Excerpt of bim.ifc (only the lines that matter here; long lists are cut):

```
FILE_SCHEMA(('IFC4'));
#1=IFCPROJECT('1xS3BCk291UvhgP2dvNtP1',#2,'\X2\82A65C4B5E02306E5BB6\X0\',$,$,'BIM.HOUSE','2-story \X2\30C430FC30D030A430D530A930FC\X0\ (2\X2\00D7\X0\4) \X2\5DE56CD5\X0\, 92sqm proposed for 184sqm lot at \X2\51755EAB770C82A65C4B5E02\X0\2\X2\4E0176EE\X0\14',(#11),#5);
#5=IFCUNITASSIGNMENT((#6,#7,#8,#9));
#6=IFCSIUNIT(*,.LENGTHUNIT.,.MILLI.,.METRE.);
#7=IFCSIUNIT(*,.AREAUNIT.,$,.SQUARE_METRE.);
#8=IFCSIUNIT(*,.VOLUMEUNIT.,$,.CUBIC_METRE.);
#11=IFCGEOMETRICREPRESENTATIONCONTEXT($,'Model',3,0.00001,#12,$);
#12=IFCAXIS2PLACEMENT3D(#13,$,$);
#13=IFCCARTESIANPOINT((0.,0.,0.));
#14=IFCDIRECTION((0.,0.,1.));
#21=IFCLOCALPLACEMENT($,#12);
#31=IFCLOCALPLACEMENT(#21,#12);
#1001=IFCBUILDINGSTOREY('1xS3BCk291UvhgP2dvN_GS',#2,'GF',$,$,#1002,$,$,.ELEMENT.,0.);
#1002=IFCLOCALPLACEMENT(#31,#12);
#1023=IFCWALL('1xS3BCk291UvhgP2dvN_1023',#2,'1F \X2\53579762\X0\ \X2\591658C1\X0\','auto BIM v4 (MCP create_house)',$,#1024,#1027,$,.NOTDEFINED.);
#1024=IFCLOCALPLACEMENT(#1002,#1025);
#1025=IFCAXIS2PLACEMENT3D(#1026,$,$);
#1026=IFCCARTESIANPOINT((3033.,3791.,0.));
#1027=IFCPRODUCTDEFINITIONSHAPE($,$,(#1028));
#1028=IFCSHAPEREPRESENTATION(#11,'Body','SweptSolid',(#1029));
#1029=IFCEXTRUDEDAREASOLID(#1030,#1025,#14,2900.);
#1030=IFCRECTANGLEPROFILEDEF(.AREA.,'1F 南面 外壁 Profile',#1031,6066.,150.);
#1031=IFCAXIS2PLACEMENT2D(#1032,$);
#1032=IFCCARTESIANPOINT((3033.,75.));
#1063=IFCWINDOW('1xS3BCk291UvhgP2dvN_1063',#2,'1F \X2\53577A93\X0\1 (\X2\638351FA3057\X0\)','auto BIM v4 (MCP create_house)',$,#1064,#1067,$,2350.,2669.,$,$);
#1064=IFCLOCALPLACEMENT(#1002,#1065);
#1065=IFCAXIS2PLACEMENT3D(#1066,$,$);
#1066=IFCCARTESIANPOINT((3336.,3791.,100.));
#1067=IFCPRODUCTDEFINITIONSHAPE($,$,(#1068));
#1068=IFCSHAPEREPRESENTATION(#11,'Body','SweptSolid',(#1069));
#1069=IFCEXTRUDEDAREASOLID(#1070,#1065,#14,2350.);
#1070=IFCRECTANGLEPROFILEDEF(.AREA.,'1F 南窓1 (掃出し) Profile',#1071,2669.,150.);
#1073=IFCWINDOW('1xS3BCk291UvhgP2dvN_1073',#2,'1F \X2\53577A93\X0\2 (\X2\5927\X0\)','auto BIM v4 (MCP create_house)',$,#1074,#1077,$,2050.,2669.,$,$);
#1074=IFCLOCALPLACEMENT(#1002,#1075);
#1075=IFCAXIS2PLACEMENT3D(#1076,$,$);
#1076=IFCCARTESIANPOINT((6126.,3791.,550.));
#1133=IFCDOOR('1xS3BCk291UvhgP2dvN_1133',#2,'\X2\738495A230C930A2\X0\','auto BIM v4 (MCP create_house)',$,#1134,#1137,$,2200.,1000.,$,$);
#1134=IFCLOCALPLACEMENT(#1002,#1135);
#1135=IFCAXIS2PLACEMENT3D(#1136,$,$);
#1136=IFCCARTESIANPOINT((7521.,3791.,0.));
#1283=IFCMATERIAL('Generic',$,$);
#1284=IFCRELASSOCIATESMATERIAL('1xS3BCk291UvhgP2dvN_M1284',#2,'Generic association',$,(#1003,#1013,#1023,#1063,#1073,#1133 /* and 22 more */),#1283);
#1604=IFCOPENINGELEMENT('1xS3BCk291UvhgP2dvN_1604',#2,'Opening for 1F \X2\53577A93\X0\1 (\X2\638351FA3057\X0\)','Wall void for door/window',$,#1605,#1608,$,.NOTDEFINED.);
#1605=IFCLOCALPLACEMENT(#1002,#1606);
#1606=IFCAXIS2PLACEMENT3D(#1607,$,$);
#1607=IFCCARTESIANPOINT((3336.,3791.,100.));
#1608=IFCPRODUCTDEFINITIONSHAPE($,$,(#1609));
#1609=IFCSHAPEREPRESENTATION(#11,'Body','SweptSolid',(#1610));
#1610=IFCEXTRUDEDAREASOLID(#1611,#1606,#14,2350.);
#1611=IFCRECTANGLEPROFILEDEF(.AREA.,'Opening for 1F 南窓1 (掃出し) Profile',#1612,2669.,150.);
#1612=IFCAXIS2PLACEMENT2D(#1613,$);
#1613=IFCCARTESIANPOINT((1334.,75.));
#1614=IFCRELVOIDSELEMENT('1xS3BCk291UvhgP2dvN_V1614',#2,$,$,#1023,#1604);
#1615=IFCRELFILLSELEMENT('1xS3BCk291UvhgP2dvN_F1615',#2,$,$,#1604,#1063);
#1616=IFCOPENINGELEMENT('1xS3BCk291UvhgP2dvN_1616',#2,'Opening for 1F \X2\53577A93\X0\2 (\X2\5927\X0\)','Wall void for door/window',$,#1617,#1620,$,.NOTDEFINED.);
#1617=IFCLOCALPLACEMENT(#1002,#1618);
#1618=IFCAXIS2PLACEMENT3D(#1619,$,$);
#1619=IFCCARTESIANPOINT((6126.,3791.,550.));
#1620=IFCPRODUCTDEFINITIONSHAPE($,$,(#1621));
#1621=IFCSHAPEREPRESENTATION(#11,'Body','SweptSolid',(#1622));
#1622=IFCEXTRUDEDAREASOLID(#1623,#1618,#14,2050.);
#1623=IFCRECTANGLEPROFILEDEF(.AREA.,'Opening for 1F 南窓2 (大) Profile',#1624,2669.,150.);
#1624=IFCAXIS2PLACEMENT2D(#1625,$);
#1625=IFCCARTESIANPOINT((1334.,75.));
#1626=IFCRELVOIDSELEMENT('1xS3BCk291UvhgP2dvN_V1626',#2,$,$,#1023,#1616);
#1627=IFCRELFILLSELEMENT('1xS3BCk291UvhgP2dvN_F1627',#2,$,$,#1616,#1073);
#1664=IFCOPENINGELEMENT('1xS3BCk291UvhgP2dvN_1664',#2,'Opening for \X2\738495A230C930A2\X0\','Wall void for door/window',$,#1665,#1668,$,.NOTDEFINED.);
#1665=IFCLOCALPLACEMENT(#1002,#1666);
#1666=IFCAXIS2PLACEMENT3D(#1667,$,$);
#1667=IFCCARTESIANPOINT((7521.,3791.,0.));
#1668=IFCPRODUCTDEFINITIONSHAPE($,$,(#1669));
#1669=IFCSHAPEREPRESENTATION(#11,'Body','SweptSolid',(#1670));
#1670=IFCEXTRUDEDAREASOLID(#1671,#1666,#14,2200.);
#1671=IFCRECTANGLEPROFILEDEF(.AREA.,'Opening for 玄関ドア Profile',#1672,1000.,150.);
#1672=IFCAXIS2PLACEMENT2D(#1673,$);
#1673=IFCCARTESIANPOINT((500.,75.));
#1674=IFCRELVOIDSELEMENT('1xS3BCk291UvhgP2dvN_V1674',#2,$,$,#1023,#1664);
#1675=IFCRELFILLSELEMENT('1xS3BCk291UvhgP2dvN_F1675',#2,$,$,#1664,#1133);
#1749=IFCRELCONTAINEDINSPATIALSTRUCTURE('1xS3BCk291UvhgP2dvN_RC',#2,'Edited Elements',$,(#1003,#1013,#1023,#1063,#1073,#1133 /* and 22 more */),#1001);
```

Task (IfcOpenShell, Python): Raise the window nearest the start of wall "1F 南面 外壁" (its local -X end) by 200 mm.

```python
import numpy as np
import ifcopenshell
import ifcopenshell.api.geometry
import ifcopenshell.util.placement
import ifcopenshell.util.unit

model = ifcopenshell.open("bim.ifc")
unit_scale = ifcopenshell.util.unit.calculate_unit_scale(model)

window = model.by_guid("1xS3BCk291UvhgP2dvN_1063")
opening = window.FillsVoids[0].RelatingOpeningElement
dz = 0.2 / unit_scale

shift = np.array([0.0, 0.0, dz])
# The window is not placed relative to its opening, so move both.
for product in (opening, window):
    matrix = ifcopenshell.util.placement.get_local_placement(product.ObjectPlacement)
    matrix[:3, 3] += shift
    ifcopenshell.api.geometry.edit_object_placement(model, product=product, matrix=matrix, is_si=False)

print(f"moved by {dz * unit_scale:+.3f} m")

model.write("bim-out.ifc")
```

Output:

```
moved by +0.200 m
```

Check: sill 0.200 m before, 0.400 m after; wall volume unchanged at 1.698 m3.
